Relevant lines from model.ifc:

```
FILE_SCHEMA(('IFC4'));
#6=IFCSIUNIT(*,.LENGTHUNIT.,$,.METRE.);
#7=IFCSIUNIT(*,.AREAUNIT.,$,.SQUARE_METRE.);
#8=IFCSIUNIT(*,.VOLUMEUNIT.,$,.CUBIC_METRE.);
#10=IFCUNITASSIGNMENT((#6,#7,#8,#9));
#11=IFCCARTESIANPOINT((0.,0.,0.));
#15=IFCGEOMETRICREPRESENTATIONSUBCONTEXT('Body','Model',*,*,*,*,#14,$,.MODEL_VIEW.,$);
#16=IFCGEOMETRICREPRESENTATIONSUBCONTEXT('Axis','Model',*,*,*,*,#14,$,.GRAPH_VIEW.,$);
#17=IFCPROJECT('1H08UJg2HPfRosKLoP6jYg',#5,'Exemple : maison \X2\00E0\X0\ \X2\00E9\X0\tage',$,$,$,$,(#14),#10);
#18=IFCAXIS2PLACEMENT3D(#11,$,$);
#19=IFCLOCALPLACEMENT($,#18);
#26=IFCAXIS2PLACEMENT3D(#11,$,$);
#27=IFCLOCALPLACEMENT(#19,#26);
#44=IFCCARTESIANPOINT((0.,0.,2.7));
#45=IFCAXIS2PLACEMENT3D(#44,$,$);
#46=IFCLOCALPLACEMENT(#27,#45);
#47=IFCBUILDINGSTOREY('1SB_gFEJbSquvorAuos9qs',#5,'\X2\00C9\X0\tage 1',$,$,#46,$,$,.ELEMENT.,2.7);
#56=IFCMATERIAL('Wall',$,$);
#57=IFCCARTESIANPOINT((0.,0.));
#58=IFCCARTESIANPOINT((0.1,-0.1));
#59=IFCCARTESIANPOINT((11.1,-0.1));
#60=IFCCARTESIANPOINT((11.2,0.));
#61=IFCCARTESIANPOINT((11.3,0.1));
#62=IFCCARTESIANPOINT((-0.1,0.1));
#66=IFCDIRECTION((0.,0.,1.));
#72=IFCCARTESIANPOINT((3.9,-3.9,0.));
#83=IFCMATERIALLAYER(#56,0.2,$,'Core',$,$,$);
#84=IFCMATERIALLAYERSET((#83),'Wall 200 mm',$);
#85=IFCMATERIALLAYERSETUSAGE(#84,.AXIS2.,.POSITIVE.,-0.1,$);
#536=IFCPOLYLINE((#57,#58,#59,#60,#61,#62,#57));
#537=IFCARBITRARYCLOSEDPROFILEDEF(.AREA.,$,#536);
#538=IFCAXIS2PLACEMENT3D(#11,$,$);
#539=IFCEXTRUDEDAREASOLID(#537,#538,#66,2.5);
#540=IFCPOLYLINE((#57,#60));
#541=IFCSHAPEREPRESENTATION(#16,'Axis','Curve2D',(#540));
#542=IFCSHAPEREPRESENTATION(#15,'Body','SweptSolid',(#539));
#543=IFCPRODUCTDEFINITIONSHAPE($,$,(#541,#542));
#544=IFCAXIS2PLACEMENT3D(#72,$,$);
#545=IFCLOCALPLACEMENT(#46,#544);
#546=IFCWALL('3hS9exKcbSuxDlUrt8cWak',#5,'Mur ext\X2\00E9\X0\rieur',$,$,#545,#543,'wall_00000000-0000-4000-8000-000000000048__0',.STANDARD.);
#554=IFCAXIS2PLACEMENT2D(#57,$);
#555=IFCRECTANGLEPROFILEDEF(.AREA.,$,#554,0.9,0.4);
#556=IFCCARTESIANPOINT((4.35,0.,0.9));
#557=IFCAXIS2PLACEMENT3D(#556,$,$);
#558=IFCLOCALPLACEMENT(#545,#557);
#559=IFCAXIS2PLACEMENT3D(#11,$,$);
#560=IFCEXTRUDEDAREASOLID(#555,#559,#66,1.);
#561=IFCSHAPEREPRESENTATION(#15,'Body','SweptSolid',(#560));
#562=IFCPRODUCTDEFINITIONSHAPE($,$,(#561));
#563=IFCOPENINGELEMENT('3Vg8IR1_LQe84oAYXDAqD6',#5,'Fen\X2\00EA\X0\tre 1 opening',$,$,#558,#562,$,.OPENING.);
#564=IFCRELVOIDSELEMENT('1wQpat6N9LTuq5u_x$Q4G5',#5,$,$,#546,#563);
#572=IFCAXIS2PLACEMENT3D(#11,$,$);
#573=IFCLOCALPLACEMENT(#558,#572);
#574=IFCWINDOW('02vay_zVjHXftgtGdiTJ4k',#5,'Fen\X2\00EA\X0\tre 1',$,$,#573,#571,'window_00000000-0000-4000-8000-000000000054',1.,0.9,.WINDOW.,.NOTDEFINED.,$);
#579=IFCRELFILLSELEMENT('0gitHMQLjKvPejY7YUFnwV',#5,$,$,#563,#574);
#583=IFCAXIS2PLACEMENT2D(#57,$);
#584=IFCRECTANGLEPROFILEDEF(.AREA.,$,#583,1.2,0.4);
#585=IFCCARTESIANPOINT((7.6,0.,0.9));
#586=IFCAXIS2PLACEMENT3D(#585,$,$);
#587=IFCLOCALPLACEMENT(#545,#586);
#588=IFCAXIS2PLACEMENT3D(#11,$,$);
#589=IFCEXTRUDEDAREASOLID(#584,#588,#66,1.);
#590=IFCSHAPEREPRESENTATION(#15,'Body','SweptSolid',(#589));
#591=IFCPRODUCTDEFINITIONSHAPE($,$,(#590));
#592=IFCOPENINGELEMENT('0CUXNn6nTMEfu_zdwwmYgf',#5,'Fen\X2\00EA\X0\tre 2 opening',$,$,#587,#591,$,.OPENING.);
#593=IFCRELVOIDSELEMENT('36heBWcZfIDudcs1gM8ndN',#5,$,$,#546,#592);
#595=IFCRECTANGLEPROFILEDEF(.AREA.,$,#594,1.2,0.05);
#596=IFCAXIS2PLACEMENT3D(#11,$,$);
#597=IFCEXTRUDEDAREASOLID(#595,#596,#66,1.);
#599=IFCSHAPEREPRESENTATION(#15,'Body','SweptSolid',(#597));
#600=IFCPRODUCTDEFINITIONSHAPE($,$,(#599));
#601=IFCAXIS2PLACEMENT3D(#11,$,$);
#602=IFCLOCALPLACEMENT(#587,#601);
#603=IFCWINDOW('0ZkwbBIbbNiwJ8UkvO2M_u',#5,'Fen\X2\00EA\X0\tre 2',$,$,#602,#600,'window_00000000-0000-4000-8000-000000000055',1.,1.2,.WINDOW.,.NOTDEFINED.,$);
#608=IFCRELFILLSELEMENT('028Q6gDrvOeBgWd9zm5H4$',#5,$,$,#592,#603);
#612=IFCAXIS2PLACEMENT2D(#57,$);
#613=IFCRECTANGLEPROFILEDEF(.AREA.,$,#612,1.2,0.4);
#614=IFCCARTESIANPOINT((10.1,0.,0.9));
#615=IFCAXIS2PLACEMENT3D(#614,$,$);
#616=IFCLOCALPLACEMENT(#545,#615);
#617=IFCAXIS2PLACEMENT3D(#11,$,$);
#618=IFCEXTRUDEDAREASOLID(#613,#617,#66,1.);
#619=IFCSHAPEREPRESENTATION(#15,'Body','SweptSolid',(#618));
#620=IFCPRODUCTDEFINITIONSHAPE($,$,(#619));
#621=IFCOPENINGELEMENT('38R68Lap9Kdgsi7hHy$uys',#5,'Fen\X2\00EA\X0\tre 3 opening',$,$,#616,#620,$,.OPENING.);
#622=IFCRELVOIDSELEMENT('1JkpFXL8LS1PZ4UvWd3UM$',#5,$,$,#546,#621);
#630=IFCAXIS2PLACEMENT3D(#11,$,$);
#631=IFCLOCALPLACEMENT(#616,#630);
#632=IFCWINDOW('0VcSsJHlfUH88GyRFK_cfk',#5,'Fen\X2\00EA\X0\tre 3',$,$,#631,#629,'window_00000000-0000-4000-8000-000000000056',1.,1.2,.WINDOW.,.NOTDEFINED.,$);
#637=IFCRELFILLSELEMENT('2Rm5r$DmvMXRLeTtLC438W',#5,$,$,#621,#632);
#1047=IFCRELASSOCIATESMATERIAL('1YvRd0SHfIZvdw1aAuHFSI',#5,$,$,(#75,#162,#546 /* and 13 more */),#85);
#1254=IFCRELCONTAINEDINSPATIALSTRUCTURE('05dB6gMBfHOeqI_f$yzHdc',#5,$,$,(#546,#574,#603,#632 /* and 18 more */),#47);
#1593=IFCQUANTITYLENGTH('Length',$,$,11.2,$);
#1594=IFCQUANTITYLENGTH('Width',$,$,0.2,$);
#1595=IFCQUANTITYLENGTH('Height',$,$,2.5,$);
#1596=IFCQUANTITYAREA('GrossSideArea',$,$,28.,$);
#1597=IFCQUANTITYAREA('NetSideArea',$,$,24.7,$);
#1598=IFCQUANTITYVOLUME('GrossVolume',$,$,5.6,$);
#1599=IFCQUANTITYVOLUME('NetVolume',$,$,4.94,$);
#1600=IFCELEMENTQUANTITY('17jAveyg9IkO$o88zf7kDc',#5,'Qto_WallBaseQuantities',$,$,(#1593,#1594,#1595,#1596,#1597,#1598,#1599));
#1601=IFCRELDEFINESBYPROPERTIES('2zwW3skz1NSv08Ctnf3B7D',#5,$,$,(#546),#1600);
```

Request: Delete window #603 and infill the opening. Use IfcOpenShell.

```python
import ifcopenshell
import ifcopenshell.api.feature
import ifcopenshell.api.pset
import ifcopenshell.api.root
import ifcopenshell.geom
import ifcopenshell.util.element
import ifcopenshell.util.shape
import ifcopenshell.util.unit

model = ifcopenshell.open("model.ifc")
area_scale = ifcopenshell.util.unit.calculate_unit_scale(model, "AREAUNIT")
volume_scale = ifcopenshell.util.unit.calculate_unit_scale(model, "VOLUMEUNIT")
settings = ifcopenshell.geom.settings()


def volume(element):
    """Net volume in cubic metres, openings subtracted."""
    shape = ifcopenshell.geom.create_shape(settings, element)
    return ifcopenshell.util.shape.get_volume(shape.geometry)


window = model.by_guid("0ZkwbBIbbNiwJ8UkvO2M_u")
opening = window.FillsVoids[0].RelatingOpeningElement
wall = opening.VoidsElements[0].RelatingBuildingElement
before = volume(wall)

ifcopenshell.api.root.remove_product(model, product=window)
ifcopenshell.api.feature.remove_feature(model, feature=opening)

after = volume(wall)
thickness = 0.2  # wall thickness in metres

# Update the wall's stored quantities.
qto = model.by_id(ifcopenshell.util.element.get_pset(wall, "Qto_WallBaseQuantities", should_inherit=False)["id"])
ifcopenshell.api.pset.edit_qto(model, qto=qto, properties={
    "NetSideArea": after / thickness / area_scale,
    "NetVolume": after / volume_scale,
})

print(f"wall volume {before:.3f} -> {after:.3f} m3")

model.write("model_v2.ifc")
```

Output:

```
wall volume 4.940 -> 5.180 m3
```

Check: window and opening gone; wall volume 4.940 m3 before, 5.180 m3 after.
